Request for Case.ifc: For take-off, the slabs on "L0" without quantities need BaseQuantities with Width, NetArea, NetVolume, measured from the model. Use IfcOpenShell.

First a look at what the model holds.

```python
import ifcopenshell
import ifcopenshell.util.element
import ifcopenshell.util.unit

model = ifcopenshell.open("Case.ifc")
print(model.schema)
for unit_type in ("LENGTHUNIT", "AREAUNIT", "VOLUMEUNIT"):
    print(unit_type, ifcopenshell.util.unit.calculate_unit_scale(model, unit_type))
storey = next(s for s in model.by_type("IfcBuildingStorey") if s.Name == "L0")
slabs = [e for e in ifcopenshell.util.element.get_decomposition(storey) if e.is_a("IfcSlab")]
for e in sorted(slabs, key=lambda e: e.id()):
    print(e.id(), e.is_a(), e.Name, list(ifcopenshell.util.element.get_psets(e, qtos_only=True)), sep=" | ")
```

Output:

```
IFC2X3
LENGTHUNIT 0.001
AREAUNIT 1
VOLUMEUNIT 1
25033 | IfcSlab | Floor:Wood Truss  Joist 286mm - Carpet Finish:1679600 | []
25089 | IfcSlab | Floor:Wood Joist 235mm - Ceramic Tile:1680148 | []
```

```python
import ifcopenshell
import ifcopenshell.api.pset
import ifcopenshell.geom
import ifcopenshell.util.element
import ifcopenshell.util.shape
import ifcopenshell.util.unit

model = ifcopenshell.open("Case.ifc")
unit_scale = ifcopenshell.util.unit.calculate_unit_scale(model)
area_scale = ifcopenshell.util.unit.calculate_unit_scale(model, "AREAUNIT")
volume_scale = ifcopenshell.util.unit.calculate_unit_scale(model, "VOLUMEUNIT")
settings = ifcopenshell.geom.settings()

storey = next(s for s in model.by_type("IfcBuildingStorey") if s.Name == "L0")
slabs = [e for e in ifcopenshell.util.element.get_decomposition(storey) if e.is_a("IfcSlab")]

for e in sorted(slabs, key=lambda e: e.id()):
    if ifcopenshell.util.element.get_psets(e, qtos_only=True, should_inherit=False):
        continue
    # Geometry comes back in metres, in the element's own axes.
    shape = ifcopenshell.geom.create_shape(settings, e)
    values = {
        "Width": ifcopenshell.util.shape.get_z(shape.geometry) / unit_scale,
        "NetArea": ifcopenshell.util.shape.get_footprint_area(shape.geometry) / area_scale,
        "NetVolume": ifcopenshell.util.shape.get_volume(shape.geometry) / volume_scale,
    }
    qto = ifcopenshell.api.pset.add_qto(model, product=e, name="BaseQuantities")
    ifcopenshell.api.pset.edit_qto(model, qto=qto, properties=values)
    print(e.id(), {k: round(v, 3) for k, v in values.items()})

model.write("Case_rev.ifc")
```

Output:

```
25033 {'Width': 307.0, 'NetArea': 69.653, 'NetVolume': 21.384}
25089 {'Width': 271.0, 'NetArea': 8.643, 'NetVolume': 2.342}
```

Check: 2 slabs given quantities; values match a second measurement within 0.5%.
